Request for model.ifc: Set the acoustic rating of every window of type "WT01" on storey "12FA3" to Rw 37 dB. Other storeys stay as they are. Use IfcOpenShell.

First a look at what the model holds.

```python
import ifcopenshell
import ifcopenshell.util.element

model = ifcopenshell.open("model.ifc")
print(model.schema)
storey = next(s for s in model.by_type("IfcBuildingStorey") if s.Name == "12FA3")
windows = [e for e in ifcopenshell.util.element.get_decomposition(storey) if e.is_a("IfcWindow")]
seen = {}
for e in windows:
    element_type = ifcopenshell.util.element.get_type(e)
    key = (element_type.Name if element_type != e and element_type else None, ifcopenshell.util.element.get_pset(e, "Pset_WindowCommon", "AcousticRating"))
    seen[key] = seen.get(key, 0) + 1
for (name, value), count in sorted(seen.items(), key=str):
    print(count, "x", name, "|", value)
```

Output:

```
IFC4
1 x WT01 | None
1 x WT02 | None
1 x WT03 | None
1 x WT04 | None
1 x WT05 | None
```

```python
import ifcopenshell
import ifcopenshell.api.pset
import ifcopenshell.util.element

model = ifcopenshell.open("model.ifc")

storey = next(s for s in model.by_type("IfcBuildingStorey") if s.Name == "12FA3")
windows = [e for e in ifcopenshell.util.element.get_decomposition(storey) if e.is_a("IfcWindow")]

count = 0
for e in windows:
    element_type = ifcopenshell.util.element.get_type(e)
    if element_type in (None, e) or element_type.Name != "WT01":
        continue
    # add_pset returns the element's existing set when there is one.
    pset = ifcopenshell.api.pset.add_pset(model, product=e, name="Pset_WindowCommon")
    ifcopenshell.api.pset.edit_pset(model, pset=pset, properties={"AcousticRating": "Rw 37 dB"})
    count += 1

print(count, "windows updated")

model.write("model-out.ifc")
```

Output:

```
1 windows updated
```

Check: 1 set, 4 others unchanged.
